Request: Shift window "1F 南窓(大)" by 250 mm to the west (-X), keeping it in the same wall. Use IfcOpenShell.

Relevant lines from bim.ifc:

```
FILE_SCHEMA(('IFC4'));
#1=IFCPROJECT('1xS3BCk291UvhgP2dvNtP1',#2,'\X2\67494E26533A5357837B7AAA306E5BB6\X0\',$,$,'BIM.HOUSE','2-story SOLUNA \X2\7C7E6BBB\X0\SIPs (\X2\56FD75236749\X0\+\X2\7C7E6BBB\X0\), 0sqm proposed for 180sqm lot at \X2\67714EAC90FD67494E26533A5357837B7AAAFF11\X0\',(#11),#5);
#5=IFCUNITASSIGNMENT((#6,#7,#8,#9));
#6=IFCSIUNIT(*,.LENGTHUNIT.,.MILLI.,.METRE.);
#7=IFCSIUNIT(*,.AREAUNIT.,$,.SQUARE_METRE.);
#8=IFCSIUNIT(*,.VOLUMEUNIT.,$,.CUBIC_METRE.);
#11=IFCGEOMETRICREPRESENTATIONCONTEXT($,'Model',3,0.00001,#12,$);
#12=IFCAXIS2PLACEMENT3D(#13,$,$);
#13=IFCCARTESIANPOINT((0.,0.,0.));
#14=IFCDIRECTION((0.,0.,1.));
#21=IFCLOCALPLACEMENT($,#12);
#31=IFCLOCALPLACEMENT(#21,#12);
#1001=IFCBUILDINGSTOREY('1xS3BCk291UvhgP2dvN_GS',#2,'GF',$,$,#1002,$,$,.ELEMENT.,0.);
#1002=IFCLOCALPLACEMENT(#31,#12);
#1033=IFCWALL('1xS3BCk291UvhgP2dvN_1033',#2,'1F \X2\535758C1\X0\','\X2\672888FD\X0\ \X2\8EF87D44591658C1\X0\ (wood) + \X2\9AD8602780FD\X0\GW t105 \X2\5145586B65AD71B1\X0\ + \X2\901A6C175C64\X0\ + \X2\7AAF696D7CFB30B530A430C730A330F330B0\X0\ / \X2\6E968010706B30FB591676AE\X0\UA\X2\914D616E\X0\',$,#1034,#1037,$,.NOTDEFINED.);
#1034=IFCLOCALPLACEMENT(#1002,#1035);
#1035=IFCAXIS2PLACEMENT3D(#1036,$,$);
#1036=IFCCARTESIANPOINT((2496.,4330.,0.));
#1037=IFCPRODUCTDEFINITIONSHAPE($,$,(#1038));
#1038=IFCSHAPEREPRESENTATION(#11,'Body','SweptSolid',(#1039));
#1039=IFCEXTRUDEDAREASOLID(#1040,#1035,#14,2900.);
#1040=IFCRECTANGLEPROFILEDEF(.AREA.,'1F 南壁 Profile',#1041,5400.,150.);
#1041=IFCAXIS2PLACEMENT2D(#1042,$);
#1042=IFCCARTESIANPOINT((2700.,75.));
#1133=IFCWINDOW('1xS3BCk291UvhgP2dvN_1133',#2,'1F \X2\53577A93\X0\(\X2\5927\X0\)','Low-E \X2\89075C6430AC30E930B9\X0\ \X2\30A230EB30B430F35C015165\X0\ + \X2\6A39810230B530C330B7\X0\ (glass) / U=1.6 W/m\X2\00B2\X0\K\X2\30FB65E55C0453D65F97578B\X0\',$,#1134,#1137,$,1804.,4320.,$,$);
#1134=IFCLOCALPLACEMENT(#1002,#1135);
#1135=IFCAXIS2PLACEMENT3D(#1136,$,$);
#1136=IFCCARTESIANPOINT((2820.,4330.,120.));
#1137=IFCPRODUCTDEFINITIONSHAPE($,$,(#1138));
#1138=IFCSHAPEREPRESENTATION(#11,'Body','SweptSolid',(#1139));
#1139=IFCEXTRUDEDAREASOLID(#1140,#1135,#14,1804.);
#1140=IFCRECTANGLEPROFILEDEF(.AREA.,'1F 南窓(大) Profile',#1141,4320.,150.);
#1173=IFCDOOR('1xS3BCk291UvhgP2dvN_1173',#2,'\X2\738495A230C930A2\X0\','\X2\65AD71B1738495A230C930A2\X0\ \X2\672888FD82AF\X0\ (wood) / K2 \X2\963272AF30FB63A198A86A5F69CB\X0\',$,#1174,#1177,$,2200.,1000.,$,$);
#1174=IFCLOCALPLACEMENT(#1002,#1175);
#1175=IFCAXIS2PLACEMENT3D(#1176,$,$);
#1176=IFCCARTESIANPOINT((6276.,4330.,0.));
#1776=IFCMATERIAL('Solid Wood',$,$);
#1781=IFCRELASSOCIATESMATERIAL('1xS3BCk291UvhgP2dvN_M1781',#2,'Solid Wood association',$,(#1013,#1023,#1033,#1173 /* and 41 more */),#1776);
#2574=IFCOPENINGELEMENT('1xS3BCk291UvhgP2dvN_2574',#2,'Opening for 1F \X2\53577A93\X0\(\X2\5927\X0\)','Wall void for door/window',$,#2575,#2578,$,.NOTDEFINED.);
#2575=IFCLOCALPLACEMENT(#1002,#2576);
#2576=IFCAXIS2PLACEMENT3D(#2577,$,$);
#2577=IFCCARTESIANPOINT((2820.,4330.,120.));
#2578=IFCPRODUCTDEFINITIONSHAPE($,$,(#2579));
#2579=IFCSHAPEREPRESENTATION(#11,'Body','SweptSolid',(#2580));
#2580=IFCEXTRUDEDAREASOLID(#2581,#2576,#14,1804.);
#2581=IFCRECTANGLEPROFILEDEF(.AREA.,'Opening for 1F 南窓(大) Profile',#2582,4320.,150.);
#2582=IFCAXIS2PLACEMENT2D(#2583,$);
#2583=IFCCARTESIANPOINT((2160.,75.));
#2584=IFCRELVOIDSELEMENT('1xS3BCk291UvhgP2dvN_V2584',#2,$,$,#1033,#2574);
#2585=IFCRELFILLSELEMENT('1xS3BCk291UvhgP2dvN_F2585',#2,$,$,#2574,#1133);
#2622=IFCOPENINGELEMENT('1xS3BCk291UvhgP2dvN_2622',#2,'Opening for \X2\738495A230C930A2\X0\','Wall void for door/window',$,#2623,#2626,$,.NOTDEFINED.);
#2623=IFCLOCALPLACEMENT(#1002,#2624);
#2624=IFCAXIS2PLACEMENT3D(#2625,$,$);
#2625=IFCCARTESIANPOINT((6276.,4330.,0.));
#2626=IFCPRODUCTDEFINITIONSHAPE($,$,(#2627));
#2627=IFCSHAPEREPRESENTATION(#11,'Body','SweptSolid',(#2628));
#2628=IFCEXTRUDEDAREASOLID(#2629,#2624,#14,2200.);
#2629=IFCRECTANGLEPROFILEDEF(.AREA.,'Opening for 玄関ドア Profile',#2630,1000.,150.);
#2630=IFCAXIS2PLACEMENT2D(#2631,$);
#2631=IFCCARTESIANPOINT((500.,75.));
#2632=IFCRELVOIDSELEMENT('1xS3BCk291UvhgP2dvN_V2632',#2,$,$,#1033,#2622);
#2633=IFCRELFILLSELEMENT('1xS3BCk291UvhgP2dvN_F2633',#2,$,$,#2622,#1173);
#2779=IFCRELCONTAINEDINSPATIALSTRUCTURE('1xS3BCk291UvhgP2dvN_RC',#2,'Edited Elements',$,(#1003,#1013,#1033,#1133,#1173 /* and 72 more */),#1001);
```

```python
import ifcopenshell
import ifcopenshell.api.geometry
import ifcopenshell.util.placement
import ifcopenshell.util.unit

model = ifcopenshell.open("bim.ifc")
unit_scale = ifcopenshell.util.unit.calculate_unit_scale(model)

window = model.by_id(1133)
opening = window.FillsVoids[0].RelatingOpeningElement
wall = opening.VoidsElements[0].RelatingBuildingElement

wall_matrix = ifcopenshell.util.placement.get_local_placement(wall.ObjectPlacement)
shift = wall_matrix[:3, 0] * -0.25 / unit_scale
before = ifcopenshell.util.placement.get_local_placement(window.ObjectPlacement)[:3, 3].copy()

# The window is not placed relative to its opening, so move both.
for product in (opening, window):
    matrix = ifcopenshell.util.placement.get_local_placement(product.ObjectPlacement)
    matrix[:3, 3] += shift
    ifcopenshell.api.geometry.edit_object_placement(model, product=product, matrix=matrix, is_si=False)

after = ifcopenshell.util.placement.get_local_placement(window.ObjectPlacement)[:3, 3]
print("window moved by", (after - before).round(3) + 0.0)

model.write("bim-out.ifc")
```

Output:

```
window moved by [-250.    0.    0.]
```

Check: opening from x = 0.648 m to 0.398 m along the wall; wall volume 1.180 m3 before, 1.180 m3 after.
